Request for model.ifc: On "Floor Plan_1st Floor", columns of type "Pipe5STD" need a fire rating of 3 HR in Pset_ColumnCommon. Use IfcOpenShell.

First a look at what the model holds.

```python
import ifcopenshell
import ifcopenshell.util.element

model = ifcopenshell.open("model.ifc")
print(model.schema)
storey = next(s for s in model.by_type("IfcBuildingStorey") if s.Name == "Floor Plan_1st Floor")
columns = [e for e in ifcopenshell.util.element.get_decomposition(storey) if e.is_a("IfcColumn")]
seen = {}
for e in columns:
    element_type = ifcopenshell.util.element.get_type(e)
    key = (element_type.Name if element_type != e and element_type else None, ifcopenshell.util.element.get_pset(e, "Pset_ColumnCommon", "FireRating"))
    seen[key] = seen.get(key, 0) + 1
for (name, value), count in sorted(seen.items(), key=str):
    print(count, "x", name, "|", value)
```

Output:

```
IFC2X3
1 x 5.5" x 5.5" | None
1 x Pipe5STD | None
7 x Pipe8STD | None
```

```python
import ifcopenshell
import ifcopenshell.api.pset
import ifcopenshell.util.element

model = ifcopenshell.open("model.ifc")

storey = next(s for s in model.by_type("IfcBuildingStorey") if s.Name == "Floor Plan_1st Floor")
columns = [e for e in ifcopenshell.util.element.get_decomposition(storey) if e.is_a("IfcColumn")]

count = 0
for e in columns:
    element_type = ifcopenshell.util.element.get_type(e)
    if element_type in (None, e) or element_type.Name != "Pipe5STD":
        continue
    # add_pset returns the element's existing set when there is one.
    pset = ifcopenshell.api.pset.add_pset(model, product=e, name="Pset_ColumnCommon")
    ifcopenshell.api.pset.edit_pset(model, pset=pset, properties={"FireRating": "3 HR"})
    count += 1

print(count, "columns updated")

model.write("model_edited.ifc")
```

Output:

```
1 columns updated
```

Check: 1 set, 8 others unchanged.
